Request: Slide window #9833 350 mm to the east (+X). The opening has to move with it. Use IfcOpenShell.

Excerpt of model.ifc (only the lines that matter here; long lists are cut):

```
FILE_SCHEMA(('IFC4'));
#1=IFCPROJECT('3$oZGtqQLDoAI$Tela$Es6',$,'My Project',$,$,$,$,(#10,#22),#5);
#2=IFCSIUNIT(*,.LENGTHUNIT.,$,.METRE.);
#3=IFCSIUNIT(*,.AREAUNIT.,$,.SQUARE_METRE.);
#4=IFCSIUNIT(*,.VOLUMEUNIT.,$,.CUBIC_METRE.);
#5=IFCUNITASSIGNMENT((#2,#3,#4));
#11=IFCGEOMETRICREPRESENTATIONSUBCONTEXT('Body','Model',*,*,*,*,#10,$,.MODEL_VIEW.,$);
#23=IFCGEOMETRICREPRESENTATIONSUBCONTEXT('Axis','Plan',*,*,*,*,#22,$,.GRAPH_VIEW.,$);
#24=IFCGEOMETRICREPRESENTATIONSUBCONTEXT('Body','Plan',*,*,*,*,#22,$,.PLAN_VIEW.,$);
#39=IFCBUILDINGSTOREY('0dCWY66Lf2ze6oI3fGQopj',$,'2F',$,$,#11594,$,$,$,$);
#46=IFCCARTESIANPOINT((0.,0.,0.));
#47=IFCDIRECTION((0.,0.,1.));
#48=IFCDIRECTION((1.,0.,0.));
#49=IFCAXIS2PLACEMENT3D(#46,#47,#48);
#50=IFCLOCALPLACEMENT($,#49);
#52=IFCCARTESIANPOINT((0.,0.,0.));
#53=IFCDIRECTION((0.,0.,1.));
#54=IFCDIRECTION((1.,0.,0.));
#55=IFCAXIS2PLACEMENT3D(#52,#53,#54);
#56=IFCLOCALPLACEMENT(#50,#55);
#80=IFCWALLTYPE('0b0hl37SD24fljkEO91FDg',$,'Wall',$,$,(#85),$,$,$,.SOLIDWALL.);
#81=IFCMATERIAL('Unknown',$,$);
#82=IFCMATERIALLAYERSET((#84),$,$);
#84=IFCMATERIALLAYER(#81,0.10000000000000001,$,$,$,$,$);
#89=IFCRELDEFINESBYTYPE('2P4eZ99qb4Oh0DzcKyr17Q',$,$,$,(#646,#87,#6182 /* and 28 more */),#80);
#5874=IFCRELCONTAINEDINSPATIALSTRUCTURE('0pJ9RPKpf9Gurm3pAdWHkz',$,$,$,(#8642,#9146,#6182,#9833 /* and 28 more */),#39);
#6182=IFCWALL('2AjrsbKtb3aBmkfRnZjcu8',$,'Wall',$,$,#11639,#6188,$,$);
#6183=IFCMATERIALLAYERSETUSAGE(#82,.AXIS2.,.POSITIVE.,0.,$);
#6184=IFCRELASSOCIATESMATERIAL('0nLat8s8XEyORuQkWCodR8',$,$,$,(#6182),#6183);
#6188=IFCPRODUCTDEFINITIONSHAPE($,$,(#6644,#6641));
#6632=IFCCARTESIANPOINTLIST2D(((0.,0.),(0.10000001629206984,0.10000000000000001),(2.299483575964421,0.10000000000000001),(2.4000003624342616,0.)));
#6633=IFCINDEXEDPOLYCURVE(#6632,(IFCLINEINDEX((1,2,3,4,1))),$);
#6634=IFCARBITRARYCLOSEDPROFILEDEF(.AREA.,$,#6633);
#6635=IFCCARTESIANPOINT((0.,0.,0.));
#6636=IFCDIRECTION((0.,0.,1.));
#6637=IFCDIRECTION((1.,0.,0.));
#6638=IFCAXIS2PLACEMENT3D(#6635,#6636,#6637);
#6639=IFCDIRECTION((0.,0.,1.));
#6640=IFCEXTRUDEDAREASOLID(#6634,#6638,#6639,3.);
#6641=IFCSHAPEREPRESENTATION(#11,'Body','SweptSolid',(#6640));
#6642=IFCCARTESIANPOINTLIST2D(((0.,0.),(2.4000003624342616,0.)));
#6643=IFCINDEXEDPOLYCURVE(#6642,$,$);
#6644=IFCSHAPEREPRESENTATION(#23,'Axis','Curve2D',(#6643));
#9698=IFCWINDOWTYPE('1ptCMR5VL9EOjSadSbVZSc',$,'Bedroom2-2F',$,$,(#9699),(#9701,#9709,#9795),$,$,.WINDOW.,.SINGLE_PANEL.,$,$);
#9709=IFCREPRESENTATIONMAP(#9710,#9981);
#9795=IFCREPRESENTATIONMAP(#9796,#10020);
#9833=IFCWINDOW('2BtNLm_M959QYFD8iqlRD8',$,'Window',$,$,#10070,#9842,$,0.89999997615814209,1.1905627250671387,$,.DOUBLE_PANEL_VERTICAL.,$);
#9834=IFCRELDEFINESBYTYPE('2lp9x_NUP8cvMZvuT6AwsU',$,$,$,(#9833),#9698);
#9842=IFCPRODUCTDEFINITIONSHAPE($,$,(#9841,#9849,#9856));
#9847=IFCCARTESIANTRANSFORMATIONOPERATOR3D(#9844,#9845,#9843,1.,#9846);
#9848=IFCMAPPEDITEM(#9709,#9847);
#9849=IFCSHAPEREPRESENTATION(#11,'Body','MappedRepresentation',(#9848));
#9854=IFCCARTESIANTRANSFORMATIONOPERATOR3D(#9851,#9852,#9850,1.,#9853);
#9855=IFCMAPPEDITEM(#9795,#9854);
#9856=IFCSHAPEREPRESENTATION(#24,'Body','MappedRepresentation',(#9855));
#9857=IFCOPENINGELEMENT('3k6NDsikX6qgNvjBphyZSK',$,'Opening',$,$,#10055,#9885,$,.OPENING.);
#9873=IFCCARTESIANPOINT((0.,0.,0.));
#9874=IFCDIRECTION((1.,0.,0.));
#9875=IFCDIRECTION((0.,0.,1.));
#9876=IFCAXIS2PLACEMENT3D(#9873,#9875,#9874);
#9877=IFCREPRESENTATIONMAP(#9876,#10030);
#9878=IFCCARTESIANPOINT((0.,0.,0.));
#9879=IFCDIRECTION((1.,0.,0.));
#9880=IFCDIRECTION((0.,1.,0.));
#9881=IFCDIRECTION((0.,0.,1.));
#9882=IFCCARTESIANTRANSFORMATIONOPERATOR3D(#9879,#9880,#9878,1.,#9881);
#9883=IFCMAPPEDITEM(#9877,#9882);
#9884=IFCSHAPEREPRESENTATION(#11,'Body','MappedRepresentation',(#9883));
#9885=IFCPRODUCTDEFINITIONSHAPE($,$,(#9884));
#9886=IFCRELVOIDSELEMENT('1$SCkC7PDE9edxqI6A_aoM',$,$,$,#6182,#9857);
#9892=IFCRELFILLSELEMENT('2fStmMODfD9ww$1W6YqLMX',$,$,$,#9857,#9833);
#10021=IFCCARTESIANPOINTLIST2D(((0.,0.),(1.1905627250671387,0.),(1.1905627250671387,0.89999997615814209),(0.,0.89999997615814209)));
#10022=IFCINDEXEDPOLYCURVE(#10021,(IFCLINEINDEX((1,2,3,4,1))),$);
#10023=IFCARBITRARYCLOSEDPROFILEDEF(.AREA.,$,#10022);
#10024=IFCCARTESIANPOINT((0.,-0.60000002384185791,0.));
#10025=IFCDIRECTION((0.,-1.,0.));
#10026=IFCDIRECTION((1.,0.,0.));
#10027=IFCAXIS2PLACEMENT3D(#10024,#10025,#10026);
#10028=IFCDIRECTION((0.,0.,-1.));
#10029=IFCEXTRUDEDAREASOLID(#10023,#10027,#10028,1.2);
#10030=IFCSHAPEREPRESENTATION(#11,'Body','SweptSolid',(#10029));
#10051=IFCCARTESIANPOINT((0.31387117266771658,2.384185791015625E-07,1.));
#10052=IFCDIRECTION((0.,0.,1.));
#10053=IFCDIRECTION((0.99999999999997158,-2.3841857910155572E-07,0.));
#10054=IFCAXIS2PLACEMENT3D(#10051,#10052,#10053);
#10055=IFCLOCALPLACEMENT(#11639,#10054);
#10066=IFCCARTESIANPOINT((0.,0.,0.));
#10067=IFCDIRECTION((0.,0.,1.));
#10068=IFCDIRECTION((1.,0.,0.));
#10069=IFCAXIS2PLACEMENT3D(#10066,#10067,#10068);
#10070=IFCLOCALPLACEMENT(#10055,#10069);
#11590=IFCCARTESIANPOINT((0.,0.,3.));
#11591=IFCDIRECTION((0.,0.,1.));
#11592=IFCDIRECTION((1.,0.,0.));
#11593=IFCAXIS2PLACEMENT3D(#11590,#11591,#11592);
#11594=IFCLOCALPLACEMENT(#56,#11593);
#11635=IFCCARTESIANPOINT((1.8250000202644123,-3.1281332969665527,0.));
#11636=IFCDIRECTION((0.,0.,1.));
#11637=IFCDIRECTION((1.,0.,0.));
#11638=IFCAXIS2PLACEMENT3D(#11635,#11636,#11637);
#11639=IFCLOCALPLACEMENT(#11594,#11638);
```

```python
import ifcopenshell
import ifcopenshell.api.geometry
import ifcopenshell.util.placement

model = ifcopenshell.open("model.ifc")

window = model.by_id(9833)
opening = window.FillsVoids[0].RelatingOpeningElement
wall = opening.VoidsElements[0].RelatingBuildingElement

wall_matrix = ifcopenshell.util.placement.get_local_placement(wall.ObjectPlacement)
shift = wall_matrix[:3, 0] * 0.35
before = ifcopenshell.util.placement.get_local_placement(window.ObjectPlacement)[:3, 3].copy()

# The window is placed relative to its opening, so it follows when the opening moves.
matrix = ifcopenshell.util.placement.get_local_placement(opening.ObjectPlacement)
matrix[:3, 3] += shift
ifcopenshell.api.geometry.edit_object_placement(
    model, product=opening, matrix=matrix, is_si=False, should_transform_children=True
)

after = ifcopenshell.util.placement.get_local_placement(window.ObjectPlacement)[:3, 3]
print("window moved by", (after - before).round(3) + 0.0)

model.write("model_edited.ifc")
```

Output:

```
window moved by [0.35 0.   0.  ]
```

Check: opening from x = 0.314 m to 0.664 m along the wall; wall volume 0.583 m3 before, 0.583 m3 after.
